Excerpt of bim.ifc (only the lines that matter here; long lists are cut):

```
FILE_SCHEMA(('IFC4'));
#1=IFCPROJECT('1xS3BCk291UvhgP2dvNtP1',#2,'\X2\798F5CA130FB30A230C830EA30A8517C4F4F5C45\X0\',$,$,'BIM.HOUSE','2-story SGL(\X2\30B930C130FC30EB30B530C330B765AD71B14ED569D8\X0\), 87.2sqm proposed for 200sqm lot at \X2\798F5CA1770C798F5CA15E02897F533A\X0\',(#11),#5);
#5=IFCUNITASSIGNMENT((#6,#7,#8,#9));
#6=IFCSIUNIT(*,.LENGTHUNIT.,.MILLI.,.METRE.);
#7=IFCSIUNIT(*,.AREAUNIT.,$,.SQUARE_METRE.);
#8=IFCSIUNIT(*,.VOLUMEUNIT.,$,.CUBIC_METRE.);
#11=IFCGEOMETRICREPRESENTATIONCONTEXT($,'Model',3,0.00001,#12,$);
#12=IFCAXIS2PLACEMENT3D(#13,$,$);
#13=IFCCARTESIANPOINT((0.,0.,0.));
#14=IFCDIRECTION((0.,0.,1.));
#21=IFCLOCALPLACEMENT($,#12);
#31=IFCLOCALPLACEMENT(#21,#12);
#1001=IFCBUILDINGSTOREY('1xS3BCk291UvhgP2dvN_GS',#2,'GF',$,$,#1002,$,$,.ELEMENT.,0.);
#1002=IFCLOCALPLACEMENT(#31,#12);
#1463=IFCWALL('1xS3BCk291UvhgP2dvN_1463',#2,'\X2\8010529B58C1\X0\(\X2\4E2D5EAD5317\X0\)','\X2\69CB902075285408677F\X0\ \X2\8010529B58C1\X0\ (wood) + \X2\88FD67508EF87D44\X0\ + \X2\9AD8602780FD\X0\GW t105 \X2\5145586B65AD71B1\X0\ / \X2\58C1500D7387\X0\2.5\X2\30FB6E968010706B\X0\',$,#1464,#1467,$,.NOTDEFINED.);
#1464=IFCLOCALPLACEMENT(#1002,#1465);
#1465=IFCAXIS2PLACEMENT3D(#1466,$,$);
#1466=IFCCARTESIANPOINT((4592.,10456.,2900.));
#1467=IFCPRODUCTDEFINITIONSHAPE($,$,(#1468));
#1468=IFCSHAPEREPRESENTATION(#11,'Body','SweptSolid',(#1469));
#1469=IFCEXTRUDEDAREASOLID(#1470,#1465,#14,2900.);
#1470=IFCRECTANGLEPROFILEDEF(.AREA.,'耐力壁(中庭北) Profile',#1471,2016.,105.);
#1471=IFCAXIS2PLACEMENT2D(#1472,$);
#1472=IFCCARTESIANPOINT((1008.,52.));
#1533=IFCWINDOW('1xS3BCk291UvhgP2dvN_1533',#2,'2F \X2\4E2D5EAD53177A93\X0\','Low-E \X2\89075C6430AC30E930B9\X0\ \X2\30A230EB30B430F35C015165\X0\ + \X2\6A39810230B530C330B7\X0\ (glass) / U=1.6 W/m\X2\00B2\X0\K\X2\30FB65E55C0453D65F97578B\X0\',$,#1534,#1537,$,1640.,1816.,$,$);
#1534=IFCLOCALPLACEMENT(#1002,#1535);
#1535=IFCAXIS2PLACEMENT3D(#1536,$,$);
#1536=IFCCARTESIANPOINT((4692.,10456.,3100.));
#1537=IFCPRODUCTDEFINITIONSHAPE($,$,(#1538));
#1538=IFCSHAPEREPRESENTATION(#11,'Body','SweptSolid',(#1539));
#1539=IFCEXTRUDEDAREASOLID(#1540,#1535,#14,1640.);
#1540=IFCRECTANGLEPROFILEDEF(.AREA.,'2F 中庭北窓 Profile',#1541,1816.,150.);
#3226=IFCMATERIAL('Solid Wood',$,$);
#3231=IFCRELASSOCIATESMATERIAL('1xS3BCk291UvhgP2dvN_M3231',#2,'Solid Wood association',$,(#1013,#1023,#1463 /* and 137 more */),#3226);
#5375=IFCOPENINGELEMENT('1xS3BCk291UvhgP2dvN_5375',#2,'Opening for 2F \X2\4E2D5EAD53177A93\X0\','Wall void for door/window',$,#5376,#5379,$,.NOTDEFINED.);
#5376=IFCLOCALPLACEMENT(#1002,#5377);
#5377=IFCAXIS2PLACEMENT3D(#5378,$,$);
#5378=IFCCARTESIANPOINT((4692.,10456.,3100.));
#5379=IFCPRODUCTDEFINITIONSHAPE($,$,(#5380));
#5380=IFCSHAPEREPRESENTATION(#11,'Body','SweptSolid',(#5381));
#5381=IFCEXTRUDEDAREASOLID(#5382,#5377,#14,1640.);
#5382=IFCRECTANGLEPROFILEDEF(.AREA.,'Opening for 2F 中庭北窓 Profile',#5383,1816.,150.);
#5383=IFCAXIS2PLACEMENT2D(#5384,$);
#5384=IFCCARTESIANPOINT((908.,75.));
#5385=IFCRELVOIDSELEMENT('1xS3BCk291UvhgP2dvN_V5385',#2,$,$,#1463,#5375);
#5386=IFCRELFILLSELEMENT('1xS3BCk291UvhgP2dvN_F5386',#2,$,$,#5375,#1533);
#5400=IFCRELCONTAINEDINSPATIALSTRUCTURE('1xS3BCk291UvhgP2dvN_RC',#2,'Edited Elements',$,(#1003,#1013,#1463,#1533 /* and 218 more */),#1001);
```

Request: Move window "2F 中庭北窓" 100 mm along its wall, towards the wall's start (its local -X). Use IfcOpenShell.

```python
import ifcopenshell
import ifcopenshell.api.geometry
import ifcopenshell.util.placement

model = ifcopenshell.open("bim.ifc")

window = model.by_id(1533)
opening = window.FillsVoids[0].RelatingOpeningElement
wall = opening.VoidsElements[0].RelatingBuildingElement

wall_matrix = ifcopenshell.util.placement.get_local_placement(wall.ObjectPlacement)
shift = wall_matrix[:3, 0] * -100.0
before = ifcopenshell.util.placement.get_local_placement(window.ObjectPlacement)[:3, 3].copy()

# The window is not placed relative to its opening, so move both.
for product in (opening, window):
    matrix = ifcopenshell.util.placement.get_local_placement(product.ObjectPlacement)
    matrix[:3, 3] += shift
    ifcopenshell.api.geometry.edit_object_placement(model, product=product, matrix=matrix, is_si=False)

after = ifcopenshell.util.placement.get_local_placement(window.ObjectPlacement)[:3, 3]
print("window moved by", (after - before).round(3) + 0.0)

model.write("bim_rev.ifc")
```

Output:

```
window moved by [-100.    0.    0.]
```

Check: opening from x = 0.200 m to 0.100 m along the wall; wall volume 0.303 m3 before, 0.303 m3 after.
